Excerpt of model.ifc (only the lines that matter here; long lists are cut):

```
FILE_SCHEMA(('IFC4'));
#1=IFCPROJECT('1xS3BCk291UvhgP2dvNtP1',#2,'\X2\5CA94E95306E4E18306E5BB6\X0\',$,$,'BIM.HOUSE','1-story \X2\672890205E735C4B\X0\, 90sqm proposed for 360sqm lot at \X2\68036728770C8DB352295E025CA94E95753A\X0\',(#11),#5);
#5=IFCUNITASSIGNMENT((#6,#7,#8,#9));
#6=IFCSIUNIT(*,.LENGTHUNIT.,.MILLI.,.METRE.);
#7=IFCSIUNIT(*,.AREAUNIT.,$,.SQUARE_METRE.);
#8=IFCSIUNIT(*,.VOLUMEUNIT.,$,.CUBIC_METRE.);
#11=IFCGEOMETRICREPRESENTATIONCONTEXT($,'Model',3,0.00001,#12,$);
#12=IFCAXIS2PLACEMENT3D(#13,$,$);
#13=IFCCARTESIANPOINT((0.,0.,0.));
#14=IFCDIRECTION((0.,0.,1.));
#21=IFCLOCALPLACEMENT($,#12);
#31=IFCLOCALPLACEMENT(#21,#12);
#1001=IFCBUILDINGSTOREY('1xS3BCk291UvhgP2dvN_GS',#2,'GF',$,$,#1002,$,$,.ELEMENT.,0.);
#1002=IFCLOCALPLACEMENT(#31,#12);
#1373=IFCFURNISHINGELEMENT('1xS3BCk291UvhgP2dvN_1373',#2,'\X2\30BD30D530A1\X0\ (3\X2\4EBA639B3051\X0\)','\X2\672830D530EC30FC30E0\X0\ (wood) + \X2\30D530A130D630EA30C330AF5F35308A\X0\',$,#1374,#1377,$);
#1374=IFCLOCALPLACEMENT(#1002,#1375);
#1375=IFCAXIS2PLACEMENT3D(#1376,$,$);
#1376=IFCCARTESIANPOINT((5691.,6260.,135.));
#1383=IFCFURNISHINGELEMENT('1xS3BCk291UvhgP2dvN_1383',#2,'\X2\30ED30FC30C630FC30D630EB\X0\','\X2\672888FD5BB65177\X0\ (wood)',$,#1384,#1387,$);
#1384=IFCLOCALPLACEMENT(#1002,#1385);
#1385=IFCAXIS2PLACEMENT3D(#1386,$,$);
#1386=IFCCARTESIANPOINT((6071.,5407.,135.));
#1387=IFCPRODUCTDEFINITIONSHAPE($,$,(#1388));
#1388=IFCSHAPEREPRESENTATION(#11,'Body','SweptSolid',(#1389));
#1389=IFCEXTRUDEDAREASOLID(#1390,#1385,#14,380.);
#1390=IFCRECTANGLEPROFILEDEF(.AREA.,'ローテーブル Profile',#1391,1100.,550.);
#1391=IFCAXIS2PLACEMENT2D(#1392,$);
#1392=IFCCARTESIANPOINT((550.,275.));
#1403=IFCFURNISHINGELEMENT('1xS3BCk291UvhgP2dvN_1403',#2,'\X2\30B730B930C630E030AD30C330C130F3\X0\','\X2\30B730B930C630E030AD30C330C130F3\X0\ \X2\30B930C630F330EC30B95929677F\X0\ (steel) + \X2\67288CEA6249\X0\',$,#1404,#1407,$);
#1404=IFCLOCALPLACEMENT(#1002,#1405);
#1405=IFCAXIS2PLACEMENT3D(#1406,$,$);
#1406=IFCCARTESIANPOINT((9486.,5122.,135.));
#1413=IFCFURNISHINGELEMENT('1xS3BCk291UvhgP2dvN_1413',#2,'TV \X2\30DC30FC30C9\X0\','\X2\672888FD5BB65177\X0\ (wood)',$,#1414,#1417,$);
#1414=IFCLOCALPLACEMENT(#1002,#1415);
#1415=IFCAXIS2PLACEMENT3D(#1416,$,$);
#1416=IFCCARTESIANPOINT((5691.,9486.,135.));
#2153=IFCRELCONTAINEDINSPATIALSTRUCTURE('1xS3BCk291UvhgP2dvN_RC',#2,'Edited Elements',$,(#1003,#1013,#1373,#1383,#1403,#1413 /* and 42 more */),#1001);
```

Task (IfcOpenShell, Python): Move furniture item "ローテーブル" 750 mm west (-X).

```python
import ifcopenshell
import ifcopenshell.api.geometry
import ifcopenshell.util.placement

model = ifcopenshell.open("model.ifc")

item = model.by_id(1383)
matrix = ifcopenshell.util.placement.get_local_placement(item.ObjectPlacement)
matrix[0, 3] -= 750.0
ifcopenshell.api.geometry.edit_object_placement(model, product=item, matrix=matrix, is_si=False)

print(ifcopenshell.util.placement.get_local_placement(item.ObjectPlacement).round(3) + 0.0)

model.write("model-out.ifc")
```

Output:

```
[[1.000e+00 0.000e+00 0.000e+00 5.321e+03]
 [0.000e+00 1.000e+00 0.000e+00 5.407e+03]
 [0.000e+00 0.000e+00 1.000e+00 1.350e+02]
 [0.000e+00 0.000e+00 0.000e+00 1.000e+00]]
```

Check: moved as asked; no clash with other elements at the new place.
